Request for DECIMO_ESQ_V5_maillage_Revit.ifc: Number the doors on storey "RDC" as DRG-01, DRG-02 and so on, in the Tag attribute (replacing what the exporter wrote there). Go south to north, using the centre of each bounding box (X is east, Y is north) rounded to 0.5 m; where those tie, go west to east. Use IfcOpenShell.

First a look at what the model holds.

```python
import ifcopenshell
import ifcopenshell.util.element
import ifcopenshell.util.placement

model = ifcopenshell.open("DECIMO_ESQ_V5_maillage_Revit.ifc")
print(model.schema)
storey = next(s for s in model.by_type("IfcBuildingStorey") if s.Name == "RDC")
doors = [e for e in ifcopenshell.util.element.get_decomposition(storey) if e.is_a("IfcDoor")]
for e in sorted(doors, key=lambda e: e.id()):
    origin = ifcopenshell.util.placement.get_local_placement(e.ObjectPlacement)[:3, 3]
    print(e.id(), e.Tag, e.Name, origin.round(2) + 0.0, sep=" | ")
```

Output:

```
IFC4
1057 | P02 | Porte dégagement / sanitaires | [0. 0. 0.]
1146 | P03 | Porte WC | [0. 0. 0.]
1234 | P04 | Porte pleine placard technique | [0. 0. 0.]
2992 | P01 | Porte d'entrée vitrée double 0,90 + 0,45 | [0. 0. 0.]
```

```python
import ifcopenshell
import ifcopenshell.geom
import ifcopenshell.util.element
import ifcopenshell.util.shape

model = ifcopenshell.open("DECIMO_ESQ_V5_maillage_Revit.ifc")
settings = ifcopenshell.geom.settings()
settings.set("use-world-coords", True)


def centre(element):
    shape = ifcopenshell.geom.create_shape(settings, element)
    return ifcopenshell.util.shape.get_bbox_centroid(shape.geometry)


storey = next(s for s in model.by_type("IfcBuildingStorey") if s.Name == "RDC")
doors = [e for e in ifcopenshell.util.element.get_decomposition(storey) if e.is_a("IfcDoor")]

# Insertion points can sit at a corner or the storey origin, so sort by the geometry (in metres).
centres = {e: centre(e) for e in doors}
doors.sort(key=lambda e: (round(centres[e][1] / 0.5), centres[e][0]))

for i, e in enumerate(doors, start=1):
    number = f"DRG-{i:02d}"
    e.Tag = number
    print(e.id(), number)

model.write("DECIMO_ESQ_V5_maillage_Revit_v2.ifc")
```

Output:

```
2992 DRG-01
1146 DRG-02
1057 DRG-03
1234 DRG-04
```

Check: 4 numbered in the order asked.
